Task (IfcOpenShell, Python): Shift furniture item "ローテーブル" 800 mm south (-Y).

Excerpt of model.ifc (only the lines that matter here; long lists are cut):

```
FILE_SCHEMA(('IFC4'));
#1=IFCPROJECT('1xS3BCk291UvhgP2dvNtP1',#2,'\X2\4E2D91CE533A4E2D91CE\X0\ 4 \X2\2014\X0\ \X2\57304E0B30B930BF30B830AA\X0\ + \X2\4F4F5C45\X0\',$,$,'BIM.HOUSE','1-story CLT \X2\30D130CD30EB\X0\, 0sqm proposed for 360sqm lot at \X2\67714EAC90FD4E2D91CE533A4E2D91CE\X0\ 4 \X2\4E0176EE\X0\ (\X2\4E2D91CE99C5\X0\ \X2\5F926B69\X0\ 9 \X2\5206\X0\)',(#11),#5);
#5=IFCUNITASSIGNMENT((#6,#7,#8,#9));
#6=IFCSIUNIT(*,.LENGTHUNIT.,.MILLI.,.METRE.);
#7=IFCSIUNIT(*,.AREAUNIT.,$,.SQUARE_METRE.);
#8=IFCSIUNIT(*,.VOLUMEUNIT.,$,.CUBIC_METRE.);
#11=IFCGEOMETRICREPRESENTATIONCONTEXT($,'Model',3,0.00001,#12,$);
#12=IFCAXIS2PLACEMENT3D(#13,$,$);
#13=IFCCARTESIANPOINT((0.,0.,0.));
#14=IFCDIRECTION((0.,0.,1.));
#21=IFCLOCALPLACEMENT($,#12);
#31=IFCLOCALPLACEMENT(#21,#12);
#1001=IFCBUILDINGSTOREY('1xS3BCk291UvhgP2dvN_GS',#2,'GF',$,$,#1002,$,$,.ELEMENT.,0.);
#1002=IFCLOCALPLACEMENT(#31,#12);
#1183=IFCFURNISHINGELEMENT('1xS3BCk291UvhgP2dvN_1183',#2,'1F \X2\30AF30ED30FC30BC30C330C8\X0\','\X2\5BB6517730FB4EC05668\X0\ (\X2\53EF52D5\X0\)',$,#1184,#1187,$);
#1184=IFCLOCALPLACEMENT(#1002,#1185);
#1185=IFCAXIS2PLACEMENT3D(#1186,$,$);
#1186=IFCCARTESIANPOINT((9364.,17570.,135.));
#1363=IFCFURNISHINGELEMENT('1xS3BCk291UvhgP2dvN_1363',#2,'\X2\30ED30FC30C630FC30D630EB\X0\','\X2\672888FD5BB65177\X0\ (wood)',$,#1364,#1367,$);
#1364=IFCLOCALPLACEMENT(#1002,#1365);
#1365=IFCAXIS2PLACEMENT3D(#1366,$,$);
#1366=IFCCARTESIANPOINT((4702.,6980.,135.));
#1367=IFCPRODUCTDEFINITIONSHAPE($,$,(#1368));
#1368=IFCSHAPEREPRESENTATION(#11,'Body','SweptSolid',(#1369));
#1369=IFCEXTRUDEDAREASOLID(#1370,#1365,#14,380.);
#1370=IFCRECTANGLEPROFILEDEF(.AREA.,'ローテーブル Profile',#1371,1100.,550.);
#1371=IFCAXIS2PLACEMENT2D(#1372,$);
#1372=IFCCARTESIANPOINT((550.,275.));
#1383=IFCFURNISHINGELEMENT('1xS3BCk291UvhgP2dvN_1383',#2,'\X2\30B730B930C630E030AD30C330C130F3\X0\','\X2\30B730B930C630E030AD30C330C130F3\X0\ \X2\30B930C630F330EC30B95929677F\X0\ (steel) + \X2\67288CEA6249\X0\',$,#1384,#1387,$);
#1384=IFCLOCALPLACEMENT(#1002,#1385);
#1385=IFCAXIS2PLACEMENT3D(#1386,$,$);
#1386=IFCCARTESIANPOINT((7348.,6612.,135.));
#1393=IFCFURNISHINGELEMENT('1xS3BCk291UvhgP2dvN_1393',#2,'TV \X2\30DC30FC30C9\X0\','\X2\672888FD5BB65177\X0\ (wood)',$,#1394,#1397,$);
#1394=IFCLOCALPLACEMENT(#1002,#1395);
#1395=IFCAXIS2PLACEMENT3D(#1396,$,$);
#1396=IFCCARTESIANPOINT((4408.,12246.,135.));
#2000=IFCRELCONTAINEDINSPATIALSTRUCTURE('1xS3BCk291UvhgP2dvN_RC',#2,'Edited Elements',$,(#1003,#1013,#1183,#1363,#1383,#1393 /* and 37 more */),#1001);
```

```python
import ifcopenshell
import ifcopenshell.api.geometry
import ifcopenshell.util.placement
import ifcopenshell.util.unit

model = ifcopenshell.open("model.ifc")
unit_scale = ifcopenshell.util.unit.calculate_unit_scale(model)

item = model.by_id(1363)
matrix = ifcopenshell.util.placement.get_local_placement(item.ObjectPlacement)
matrix[1, 3] -= 0.8 / unit_scale
ifcopenshell.api.geometry.edit_object_placement(model, product=item, matrix=matrix, is_si=False)

print(ifcopenshell.util.placement.get_local_placement(item.ObjectPlacement).round(3) + 0.0)

model.write("model_edited.ifc")
```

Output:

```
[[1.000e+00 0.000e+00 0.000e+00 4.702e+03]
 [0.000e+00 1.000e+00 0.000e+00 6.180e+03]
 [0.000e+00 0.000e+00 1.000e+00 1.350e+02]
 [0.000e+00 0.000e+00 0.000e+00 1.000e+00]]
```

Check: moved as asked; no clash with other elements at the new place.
